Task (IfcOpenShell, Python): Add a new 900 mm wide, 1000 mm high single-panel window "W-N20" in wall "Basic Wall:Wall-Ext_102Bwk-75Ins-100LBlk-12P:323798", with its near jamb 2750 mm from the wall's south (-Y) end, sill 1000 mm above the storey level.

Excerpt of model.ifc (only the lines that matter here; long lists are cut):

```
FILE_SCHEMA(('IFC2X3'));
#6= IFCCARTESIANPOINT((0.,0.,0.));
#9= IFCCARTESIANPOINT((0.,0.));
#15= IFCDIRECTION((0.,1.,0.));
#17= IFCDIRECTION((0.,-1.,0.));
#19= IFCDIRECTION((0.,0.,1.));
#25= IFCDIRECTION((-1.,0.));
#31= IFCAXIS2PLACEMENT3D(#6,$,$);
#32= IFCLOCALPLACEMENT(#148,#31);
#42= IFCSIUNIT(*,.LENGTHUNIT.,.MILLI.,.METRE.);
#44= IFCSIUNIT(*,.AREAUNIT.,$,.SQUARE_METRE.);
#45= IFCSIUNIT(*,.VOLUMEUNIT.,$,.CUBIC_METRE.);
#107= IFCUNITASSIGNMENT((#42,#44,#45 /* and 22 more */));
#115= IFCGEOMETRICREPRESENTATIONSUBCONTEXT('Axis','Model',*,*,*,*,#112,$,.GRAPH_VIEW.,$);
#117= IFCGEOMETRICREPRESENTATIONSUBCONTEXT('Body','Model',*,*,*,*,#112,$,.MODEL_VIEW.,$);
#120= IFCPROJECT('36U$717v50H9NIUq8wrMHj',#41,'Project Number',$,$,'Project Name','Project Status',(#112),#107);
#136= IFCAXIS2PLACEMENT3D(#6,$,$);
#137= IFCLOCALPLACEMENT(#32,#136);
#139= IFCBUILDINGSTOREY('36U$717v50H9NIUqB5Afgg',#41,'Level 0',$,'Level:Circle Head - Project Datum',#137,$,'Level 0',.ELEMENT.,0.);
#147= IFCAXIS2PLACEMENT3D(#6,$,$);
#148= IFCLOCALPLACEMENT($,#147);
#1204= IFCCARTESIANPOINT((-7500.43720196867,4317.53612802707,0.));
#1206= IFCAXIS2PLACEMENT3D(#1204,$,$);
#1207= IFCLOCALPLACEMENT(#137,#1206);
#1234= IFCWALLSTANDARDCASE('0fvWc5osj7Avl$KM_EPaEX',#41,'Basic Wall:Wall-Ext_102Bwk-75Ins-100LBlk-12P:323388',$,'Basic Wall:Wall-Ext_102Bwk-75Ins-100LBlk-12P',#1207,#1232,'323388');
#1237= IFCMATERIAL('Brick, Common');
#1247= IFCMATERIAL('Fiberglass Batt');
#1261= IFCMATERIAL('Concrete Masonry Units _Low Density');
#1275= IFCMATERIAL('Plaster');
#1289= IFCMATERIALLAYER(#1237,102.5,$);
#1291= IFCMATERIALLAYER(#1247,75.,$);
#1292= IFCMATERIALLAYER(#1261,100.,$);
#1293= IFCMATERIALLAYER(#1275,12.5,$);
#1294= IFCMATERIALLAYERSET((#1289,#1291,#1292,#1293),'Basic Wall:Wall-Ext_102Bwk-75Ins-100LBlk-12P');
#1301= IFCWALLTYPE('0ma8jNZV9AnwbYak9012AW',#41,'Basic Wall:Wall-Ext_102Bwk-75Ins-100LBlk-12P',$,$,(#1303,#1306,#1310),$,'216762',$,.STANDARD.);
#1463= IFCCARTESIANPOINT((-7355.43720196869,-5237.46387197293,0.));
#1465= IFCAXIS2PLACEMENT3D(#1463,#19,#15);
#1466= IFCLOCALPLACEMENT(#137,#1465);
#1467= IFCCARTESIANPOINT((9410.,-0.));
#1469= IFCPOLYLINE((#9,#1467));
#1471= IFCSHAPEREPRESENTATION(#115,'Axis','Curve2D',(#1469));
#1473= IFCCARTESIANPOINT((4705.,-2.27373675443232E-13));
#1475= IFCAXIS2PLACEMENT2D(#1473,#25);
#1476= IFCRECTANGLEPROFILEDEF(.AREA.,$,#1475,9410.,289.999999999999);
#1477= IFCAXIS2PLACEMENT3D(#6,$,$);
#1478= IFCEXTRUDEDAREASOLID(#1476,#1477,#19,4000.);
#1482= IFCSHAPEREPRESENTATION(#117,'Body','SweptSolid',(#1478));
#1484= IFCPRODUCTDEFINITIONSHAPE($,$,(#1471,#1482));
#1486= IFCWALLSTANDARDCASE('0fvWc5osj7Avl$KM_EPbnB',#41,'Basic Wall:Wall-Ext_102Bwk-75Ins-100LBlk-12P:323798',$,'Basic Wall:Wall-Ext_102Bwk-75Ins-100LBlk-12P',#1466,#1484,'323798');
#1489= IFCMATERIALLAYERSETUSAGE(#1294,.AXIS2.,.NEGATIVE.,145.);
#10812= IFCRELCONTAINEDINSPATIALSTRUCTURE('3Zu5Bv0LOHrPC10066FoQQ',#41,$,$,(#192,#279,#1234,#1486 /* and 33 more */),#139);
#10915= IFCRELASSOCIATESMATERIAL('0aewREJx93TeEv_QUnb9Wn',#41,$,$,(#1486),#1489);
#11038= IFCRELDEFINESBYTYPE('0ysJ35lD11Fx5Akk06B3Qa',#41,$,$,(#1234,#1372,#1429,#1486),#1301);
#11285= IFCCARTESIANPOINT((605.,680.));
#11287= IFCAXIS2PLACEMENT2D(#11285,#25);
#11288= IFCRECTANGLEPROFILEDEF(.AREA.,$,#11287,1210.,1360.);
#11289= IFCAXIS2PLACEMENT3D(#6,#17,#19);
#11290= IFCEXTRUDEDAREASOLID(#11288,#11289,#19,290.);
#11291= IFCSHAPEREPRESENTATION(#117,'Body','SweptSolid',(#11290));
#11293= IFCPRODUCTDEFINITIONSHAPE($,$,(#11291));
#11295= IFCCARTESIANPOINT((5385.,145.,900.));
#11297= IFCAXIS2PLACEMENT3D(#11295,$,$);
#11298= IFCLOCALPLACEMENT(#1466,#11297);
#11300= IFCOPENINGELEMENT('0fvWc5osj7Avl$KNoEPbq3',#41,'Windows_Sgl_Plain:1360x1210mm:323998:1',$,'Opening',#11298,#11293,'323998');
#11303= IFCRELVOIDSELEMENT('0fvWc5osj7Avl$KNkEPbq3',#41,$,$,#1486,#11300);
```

```python
import numpy as np
import ifcopenshell
import ifcopenshell.api.feature
import ifcopenshell.api.geometry
import ifcopenshell.api.root
import ifcopenshell.api.spatial
import ifcopenshell.api.type
import ifcopenshell.geom
import ifcopenshell.util.element
import ifcopenshell.util.placement
import ifcopenshell.util.representation
import ifcopenshell.util.shape
import ifcopenshell.util.unit

model = ifcopenshell.open("model.ifc")
unit_scale = ifcopenshell.util.unit.calculate_unit_scale(model)
settings = ifcopenshell.geom.settings()


def volume(element):
    """Net volume in cubic metres, openings subtracted."""
    shape = ifcopenshell.geom.create_shape(settings, element)
    return ifcopenshell.util.shape.get_volume(shape.geometry)


wall = model.by_id(1486)
storey = ifcopenshell.util.element.get_container(wall, ifc_class="IfcBuildingStorey")
context = ifcopenshell.util.representation.get_context(model, "Model", "Body", "MODEL_VIEW")
before = volume(wall)

width, height, from_end, sill = 0.9, 1, 2.75, 1  # metres

# The wall runs along its own X axis, and the end named is its -X end.
wall_shape = ifcopenshell.geom.create_shape(settings, wall)
x, y, z = ifcopenshell.util.shape.get_vertices(wall_shape.geometry).T
start = x.min() + from_end
face, thickness = float(y.min()), float(y.max() - y.min())
wall_matrix = ifcopenshell.util.placement.get_local_placement(wall.ObjectPlacement)
level = ifcopenshell.util.placement.get_local_placement(storey.ObjectPlacement)[2, 3]


def in_wall(x, y):
    """Placement at x, y metres in the wall's axes, at sill height."""
    matrix = wall_matrix.copy()
    matrix[:, 3] = wall_matrix @ np.array([x / unit_scale, y / unit_scale, 0.0, 1.0])
    matrix[2, 3] = level + sill / unit_scale
    return matrix


# Opening: a box that overshoots both wall faces by 50 mm.
opening = ifcopenshell.api.root.create_entity(model, ifc_class="IfcOpeningElement")
box = ifcopenshell.api.geometry.add_wall_representation(
    model, context=context, length=width, height=height, thickness=thickness + 0.1
)
ifcopenshell.api.geometry.assign_representation(model, product=opening, representation=box)
ifcopenshell.api.geometry.edit_object_placement(model, product=opening, matrix=in_wall(start, face - 0.05), is_si=False)
ifcopenshell.api.feature.add_feature(model, feature=opening, element=wall)

window = ifcopenshell.api.root.create_entity(model, ifc_class="IfcWindow", name="W-N20")
window.OverallWidth, window.OverallHeight = width / unit_scale, height / unit_scale
body = ifcopenshell.api.geometry.add_window_representation(
    model,
    context=context,
    overall_width=window.OverallWidth,
    overall_height=window.OverallHeight,
    partition_type="SINGLE_PANEL",
)
ifcopenshell.api.geometry.assign_representation(model, product=window, representation=body)
ifcopenshell.api.spatial.assign_container(model, products=[window], relating_structure=storey)
fills = ifcopenshell.api.feature.add_filling(model, opening=opening, element=window)
fills.OwnerHistory = window.OwnerHistory  # required in IFC2X3

# IFC2X3 keeps the operation on the window style.
style = ifcopenshell.api.root.create_entity(model, ifc_class="IfcWindowStyle", name="W-N20")
style.OperationType, style.ConstructionType = "SINGLE_PANEL", "NOTDEFINED"
style.ParameterTakesPrecedence = style.Sizeable = False
ifcopenshell.api.type.assign_type(model, related_objects=[window], relating_type=style)

# Centre the window in the wall's thickness.
ifcopenshell.api.geometry.edit_object_placement(model, product=window, matrix=in_wall(start, face), is_si=False)
window_shape = ifcopenshell.geom.create_shape(settings, window)
depth = ifcopenshell.util.shape.get_vertices(window_shape.geometry)[:, 1]
offset = face + thickness / 2 - (depth.min() + depth.max()) / 2
ifcopenshell.api.geometry.edit_object_placement(model, product=window, matrix=in_wall(start, offset), is_si=False)

after = volume(wall)

print(f"wall volume {before:.3f} -> {after:.3f} m3")

model.write("model_edited.ifc")
```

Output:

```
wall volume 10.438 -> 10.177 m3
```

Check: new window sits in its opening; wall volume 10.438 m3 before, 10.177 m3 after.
